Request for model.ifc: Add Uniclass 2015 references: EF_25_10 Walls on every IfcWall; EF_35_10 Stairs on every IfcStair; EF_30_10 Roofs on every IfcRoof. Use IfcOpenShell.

First a look at what the model holds.

```python
import ifcopenshell

model = ifcopenshell.open("model.ifc")
print(model.schema)
print("classifications:", [c.Name for c in model.by_type("IfcClassification")])
for ifc_class in ("IfcDoor", "IfcRoof", "IfcStair", "IfcWall", "IfcWindow"):
    print(ifc_class, len(model.by_type(ifc_class)))
```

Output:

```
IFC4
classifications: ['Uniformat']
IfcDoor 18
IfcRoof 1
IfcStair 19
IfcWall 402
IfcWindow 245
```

```python
import ifcopenshell
import ifcopenshell.api.classification

model = ifcopenshell.open("model.ifc")

system = ifcopenshell.api.classification.add_classification(model, classification="Uniclass 2015")

codes = {
    "IfcWall": ("EF_25_10", "Walls"),
    "IfcStair": ("EF_35_10", "Stairs"),
    "IfcRoof": ("EF_30_10", "Roofs"),
}
for ifc_class, (code, name) in codes.items():
    products = model.by_type(ifc_class)
    ifcopenshell.api.classification.add_reference(
        model, products=products, classification=system, identification=code, name=name
    )
    print(code, len(products))

model.write("model_updated.ifc")
```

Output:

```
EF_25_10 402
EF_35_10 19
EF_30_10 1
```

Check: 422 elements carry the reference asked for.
